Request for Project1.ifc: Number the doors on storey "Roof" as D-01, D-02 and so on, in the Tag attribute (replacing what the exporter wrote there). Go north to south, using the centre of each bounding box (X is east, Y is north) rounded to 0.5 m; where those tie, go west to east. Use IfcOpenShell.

First a look at what the model holds.

```python
import ifcopenshell
import ifcopenshell.util.element
import ifcopenshell.util.placement

model = ifcopenshell.open("Project1.ifc")
print(model.schema)
storey = next(s for s in model.by_type("IfcBuildingStorey") if s.Name == "Roof")
doors = [e for e in ifcopenshell.util.element.get_decomposition(storey) if e.is_a("IfcDoor")]
for e in sorted(doors, key=lambda e: e.id()):
    origin = ifcopenshell.util.placement.get_local_placement(e.ObjectPlacement)[:3, 3]
    print(e.id(), e.Tag, e.Name, origin.round(2) + 0.0, sep=" | ")
```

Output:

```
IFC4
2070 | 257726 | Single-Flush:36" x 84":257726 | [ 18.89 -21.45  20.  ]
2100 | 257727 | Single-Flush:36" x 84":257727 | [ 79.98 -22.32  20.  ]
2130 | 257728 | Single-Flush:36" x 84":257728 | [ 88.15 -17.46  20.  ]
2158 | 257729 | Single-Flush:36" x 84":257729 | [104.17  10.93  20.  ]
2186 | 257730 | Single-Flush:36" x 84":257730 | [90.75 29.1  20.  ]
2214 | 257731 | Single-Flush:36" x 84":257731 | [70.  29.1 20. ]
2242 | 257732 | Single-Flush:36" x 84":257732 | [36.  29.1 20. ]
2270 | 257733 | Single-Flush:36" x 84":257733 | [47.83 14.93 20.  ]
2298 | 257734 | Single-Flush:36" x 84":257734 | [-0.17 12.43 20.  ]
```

```python
import ifcopenshell
import ifcopenshell.geom
import ifcopenshell.util.element
import ifcopenshell.util.shape

model = ifcopenshell.open("Project1.ifc")
settings = ifcopenshell.geom.settings()
settings.set("use-world-coords", True)


def centre(element):
    shape = ifcopenshell.geom.create_shape(settings, element)
    return ifcopenshell.util.shape.get_bbox_centroid(shape.geometry)


storey = next(s for s in model.by_type("IfcBuildingStorey") if s.Name == "Roof")
doors = [e for e in ifcopenshell.util.element.get_decomposition(storey) if e.is_a("IfcDoor")]

# Insertion points can sit at a corner or the storey origin, so sort by the geometry (in metres).
centres = {e: centre(e) for e in doors}
doors.sort(key=lambda e: (-round(centres[e][1] / 0.5), centres[e][0]))

for i, e in enumerate(doors, start=1):
    number = f"D-{i:02d}"
    e.Tag = number
    print(e.id(), number)

model.write("Project1_updated.ifc")
```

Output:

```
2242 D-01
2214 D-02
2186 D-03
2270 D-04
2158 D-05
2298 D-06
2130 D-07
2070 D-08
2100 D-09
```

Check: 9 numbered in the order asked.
